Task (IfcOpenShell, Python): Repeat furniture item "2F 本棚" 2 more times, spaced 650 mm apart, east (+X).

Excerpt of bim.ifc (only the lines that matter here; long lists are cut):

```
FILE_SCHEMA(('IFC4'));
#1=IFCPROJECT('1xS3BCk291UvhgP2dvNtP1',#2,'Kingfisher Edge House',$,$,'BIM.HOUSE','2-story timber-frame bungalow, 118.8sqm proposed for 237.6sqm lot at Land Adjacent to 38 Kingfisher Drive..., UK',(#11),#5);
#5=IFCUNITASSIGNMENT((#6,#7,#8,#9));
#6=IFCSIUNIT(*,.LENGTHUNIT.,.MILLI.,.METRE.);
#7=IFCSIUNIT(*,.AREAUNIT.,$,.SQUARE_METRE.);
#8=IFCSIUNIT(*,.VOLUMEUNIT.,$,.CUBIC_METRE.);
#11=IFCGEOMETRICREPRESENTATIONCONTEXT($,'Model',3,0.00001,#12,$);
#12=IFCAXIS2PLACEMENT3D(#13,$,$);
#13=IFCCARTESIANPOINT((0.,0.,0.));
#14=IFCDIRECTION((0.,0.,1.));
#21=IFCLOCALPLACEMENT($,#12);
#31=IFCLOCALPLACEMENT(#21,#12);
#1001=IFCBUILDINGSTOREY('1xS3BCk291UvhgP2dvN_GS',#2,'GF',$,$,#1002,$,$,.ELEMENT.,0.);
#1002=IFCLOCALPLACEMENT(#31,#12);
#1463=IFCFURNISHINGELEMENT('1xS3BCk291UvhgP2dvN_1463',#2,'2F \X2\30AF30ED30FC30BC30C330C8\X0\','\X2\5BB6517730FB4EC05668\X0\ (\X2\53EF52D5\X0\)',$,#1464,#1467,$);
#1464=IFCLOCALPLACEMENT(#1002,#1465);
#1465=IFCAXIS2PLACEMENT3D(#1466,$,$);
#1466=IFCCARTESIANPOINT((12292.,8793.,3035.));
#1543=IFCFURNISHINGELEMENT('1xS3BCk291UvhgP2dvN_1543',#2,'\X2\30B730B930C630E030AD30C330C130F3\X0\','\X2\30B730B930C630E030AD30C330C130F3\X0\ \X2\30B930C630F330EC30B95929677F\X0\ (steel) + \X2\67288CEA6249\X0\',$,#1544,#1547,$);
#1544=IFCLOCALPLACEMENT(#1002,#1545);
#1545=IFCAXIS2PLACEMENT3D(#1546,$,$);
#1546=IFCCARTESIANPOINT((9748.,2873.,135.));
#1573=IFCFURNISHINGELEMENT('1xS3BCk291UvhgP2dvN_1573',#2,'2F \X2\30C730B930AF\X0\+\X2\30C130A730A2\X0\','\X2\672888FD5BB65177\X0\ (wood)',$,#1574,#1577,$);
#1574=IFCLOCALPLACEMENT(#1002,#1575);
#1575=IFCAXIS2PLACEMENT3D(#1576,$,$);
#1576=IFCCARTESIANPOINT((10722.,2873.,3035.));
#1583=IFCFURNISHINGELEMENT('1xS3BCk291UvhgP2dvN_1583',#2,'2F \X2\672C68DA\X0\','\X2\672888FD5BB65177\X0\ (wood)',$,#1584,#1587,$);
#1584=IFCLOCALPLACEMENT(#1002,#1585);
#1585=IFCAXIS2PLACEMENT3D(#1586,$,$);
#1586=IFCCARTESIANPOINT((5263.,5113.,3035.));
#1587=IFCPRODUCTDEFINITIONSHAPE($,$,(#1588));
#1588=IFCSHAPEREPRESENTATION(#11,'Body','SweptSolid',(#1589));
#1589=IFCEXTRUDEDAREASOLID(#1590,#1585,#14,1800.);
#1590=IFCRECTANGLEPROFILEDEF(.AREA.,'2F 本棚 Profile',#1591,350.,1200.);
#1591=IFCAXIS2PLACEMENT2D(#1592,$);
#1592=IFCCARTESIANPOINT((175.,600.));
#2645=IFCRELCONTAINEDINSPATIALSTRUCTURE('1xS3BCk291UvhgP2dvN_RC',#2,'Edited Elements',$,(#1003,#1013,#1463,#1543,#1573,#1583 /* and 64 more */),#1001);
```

```python
import numpy as np
import ifcopenshell
import ifcopenshell.api.geometry
import ifcopenshell.api.root
import ifcopenshell.util.element
import ifcopenshell.util.placement

model = ifcopenshell.open("bim.ifc")


def reuse_history(source, copy):
    """copy_class also copies each property set's owner history, people and application; keep the originals."""
    for rel in copy.IsDefinedBy:
        if rel.is_a("IfcRelDefinesByProperties") and (history := rel.RelatingPropertyDefinition.OwnerHistory):
            rel.RelatingPropertyDefinition.OwnerHistory = source.OwnerHistory
            ifcopenshell.util.element.remove_deep2(model, history)


source = model.by_guid("1xS3BCk291UvhgP2dvN_1583")
base = ifcopenshell.util.placement.get_local_placement(source.ObjectPlacement)
step = np.array([1.0, 0.0, 0.0]) * 650.0

for i in range(1, 3):
    copy = ifcopenshell.api.root.copy_class(model, product=source)
    copy.Representation = ifcopenshell.util.element.copy_deep(
        model, source.Representation, exclude=["IfcGeometricRepresentationContext", "IfcRepresentationMap"]
    )
    reuse_history(source, copy)
    matrix = base.copy()
    matrix[:3, 3] += i * step
    print("added at", matrix[:3, 3].round(3) + 0.0)
    ifcopenshell.api.geometry.edit_object_placement(model, product=copy, matrix=matrix, is_si=False)

model.write("bim_v2.ifc")
```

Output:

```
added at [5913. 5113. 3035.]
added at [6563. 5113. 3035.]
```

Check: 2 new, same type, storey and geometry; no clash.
